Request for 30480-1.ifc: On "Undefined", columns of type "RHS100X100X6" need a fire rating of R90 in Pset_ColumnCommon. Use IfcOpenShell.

First a look at what the model holds.

```python
import ifcopenshell
import ifcopenshell.util.element

model = ifcopenshell.open("30480-1.ifc")
print(model.schema)
storey = next(s for s in model.by_type("IfcBuildingStorey") if s.Name == "Undefined")
columns = [e for e in ifcopenshell.util.element.get_decomposition(storey) if e.is_a("IfcColumn")]
seen = {}
for e in columns:
    element_type = ifcopenshell.util.element.get_type(e)
    key = (element_type.Name if element_type != e and element_type else None, ifcopenshell.util.element.get_pset(e, "Pset_ColumnCommon", "FireRating"))
    seen[key] = seen.get(key, 0) + 1
for (name, value), count in sorted(seen.items(), key=str):
    print(count, "x", name, "|", value)
```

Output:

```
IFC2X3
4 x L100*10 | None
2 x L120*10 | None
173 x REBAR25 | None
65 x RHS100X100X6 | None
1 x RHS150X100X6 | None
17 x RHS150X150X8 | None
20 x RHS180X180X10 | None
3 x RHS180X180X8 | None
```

```python
import ifcopenshell
import ifcopenshell.api.pset
import ifcopenshell.util.element

model = ifcopenshell.open("30480-1.ifc")

storey = next(s for s in model.by_type("IfcBuildingStorey") if s.Name == "Undefined")
columns = [e for e in ifcopenshell.util.element.get_decomposition(storey) if e.is_a("IfcColumn")]

count = 0
for e in columns:
    element_type = ifcopenshell.util.element.get_type(e)
    if element_type in (None, e) or element_type.Name != "RHS100X100X6":
        continue
    found = ifcopenshell.util.element.get_pset(e, "Pset_ColumnCommon", should_inherit=False)
    if found:
        pset = model.by_id(found["id"])
        if len(ifcopenshell.util.element.get_elements_by_pset(pset)) > 1:
            pset = ifcopenshell.api.pset.unshare_pset(model, products=[e], pset=pset)[0]
    else:
        pset = ifcopenshell.api.pset.add_pset(model, product=e, name="Pset_ColumnCommon")
    ifcopenshell.api.pset.edit_pset(model, pset=pset, properties={"FireRating": "R90"})
    count += 1

print(count, "columns updated")

model.write("30480-1-out.ifc")
```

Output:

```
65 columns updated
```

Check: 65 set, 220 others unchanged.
